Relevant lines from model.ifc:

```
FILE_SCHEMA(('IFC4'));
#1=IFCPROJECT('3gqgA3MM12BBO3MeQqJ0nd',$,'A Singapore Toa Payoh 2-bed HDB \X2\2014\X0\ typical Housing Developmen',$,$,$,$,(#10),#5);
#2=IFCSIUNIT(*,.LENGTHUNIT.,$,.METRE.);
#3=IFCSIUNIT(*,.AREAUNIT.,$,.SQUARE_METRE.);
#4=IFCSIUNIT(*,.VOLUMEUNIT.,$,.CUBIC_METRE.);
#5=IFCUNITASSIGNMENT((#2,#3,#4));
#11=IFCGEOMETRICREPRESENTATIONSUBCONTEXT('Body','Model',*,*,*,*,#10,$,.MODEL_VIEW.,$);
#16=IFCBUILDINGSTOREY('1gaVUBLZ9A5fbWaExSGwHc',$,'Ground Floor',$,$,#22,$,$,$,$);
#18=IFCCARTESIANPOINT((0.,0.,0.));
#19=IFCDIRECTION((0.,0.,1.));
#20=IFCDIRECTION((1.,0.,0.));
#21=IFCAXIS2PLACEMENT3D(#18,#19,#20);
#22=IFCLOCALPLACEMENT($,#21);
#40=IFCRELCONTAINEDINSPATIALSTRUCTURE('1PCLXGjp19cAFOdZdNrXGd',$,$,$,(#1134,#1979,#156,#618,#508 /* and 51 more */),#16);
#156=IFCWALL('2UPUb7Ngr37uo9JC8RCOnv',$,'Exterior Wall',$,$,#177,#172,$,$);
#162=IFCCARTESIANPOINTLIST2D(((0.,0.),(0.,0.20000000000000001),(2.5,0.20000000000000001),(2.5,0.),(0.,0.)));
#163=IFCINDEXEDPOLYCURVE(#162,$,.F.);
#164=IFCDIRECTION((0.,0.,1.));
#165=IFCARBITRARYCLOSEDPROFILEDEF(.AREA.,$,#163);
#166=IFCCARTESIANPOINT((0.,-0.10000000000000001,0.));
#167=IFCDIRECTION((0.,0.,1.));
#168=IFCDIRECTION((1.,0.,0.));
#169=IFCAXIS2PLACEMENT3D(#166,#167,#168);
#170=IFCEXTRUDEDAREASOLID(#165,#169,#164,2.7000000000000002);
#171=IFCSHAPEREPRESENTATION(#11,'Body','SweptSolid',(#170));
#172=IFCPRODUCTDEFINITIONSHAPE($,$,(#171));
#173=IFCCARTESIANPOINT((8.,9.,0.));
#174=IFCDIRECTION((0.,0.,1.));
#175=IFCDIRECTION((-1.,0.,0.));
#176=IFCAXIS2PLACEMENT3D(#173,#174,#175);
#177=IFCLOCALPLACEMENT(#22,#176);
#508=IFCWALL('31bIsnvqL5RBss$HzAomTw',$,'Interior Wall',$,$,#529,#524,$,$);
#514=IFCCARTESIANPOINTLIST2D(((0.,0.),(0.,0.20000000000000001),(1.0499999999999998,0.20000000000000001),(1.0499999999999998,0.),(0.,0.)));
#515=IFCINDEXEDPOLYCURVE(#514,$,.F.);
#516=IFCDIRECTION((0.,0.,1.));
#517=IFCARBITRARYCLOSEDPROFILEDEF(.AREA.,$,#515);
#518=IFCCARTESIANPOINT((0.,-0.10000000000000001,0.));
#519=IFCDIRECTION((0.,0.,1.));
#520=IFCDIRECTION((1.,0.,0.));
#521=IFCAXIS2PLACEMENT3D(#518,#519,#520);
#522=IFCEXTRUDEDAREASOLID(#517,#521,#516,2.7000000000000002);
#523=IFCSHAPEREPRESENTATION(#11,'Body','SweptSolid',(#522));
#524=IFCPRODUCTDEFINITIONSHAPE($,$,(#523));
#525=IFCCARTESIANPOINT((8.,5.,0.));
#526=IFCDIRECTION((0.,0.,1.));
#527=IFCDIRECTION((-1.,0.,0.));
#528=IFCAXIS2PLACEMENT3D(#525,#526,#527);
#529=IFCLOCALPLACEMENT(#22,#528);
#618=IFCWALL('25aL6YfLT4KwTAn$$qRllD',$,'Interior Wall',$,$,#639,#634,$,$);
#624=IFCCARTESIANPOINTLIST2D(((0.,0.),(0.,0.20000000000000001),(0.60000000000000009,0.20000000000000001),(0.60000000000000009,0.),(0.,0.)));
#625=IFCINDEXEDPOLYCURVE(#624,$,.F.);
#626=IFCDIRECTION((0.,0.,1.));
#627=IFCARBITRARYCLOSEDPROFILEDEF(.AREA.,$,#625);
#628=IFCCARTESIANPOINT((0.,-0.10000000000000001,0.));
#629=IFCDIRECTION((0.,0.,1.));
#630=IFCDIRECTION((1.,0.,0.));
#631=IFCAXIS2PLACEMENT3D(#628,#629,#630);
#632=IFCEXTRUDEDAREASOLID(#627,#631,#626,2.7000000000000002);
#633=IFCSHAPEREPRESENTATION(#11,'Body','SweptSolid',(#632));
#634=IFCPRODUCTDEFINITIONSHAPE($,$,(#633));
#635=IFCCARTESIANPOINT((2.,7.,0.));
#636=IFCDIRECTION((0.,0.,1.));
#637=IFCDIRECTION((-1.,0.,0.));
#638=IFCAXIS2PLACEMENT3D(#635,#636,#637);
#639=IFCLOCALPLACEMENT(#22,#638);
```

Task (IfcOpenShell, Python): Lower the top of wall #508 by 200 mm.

```python
import ifcopenshell
import ifcopenshell.geom
import ifcopenshell.util.representation
import ifcopenshell.util.shape
import ifcopenshell.util.unit

model = ifcopenshell.open("model.ifc")
unit_scale = ifcopenshell.util.unit.calculate_unit_scale(model)
settings = ifcopenshell.geom.settings()


def volume(element):
    """Net volume in cubic metres, openings subtracted."""
    shape = ifcopenshell.geom.create_shape(settings, element)
    return ifcopenshell.util.shape.get_volume(shape.geometry)


wall = model.by_guid("31bIsnvqL5RBss$HzAomTw")
before = volume(wall)

body = ifcopenshell.util.representation.get_representation(wall, "Model", "Body")
solid = body.Items[0]
old_height = solid.Depth
solid.Depth -= 0.2 / unit_scale
after = volume(wall)

print(f"height {old_height:g} -> {solid.Depth:g}, volume {before:.3f} -> {after:.3f} m3")

model.write("model_v2.ifc")
```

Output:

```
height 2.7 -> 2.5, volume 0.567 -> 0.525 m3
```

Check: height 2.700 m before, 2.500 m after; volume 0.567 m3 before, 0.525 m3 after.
